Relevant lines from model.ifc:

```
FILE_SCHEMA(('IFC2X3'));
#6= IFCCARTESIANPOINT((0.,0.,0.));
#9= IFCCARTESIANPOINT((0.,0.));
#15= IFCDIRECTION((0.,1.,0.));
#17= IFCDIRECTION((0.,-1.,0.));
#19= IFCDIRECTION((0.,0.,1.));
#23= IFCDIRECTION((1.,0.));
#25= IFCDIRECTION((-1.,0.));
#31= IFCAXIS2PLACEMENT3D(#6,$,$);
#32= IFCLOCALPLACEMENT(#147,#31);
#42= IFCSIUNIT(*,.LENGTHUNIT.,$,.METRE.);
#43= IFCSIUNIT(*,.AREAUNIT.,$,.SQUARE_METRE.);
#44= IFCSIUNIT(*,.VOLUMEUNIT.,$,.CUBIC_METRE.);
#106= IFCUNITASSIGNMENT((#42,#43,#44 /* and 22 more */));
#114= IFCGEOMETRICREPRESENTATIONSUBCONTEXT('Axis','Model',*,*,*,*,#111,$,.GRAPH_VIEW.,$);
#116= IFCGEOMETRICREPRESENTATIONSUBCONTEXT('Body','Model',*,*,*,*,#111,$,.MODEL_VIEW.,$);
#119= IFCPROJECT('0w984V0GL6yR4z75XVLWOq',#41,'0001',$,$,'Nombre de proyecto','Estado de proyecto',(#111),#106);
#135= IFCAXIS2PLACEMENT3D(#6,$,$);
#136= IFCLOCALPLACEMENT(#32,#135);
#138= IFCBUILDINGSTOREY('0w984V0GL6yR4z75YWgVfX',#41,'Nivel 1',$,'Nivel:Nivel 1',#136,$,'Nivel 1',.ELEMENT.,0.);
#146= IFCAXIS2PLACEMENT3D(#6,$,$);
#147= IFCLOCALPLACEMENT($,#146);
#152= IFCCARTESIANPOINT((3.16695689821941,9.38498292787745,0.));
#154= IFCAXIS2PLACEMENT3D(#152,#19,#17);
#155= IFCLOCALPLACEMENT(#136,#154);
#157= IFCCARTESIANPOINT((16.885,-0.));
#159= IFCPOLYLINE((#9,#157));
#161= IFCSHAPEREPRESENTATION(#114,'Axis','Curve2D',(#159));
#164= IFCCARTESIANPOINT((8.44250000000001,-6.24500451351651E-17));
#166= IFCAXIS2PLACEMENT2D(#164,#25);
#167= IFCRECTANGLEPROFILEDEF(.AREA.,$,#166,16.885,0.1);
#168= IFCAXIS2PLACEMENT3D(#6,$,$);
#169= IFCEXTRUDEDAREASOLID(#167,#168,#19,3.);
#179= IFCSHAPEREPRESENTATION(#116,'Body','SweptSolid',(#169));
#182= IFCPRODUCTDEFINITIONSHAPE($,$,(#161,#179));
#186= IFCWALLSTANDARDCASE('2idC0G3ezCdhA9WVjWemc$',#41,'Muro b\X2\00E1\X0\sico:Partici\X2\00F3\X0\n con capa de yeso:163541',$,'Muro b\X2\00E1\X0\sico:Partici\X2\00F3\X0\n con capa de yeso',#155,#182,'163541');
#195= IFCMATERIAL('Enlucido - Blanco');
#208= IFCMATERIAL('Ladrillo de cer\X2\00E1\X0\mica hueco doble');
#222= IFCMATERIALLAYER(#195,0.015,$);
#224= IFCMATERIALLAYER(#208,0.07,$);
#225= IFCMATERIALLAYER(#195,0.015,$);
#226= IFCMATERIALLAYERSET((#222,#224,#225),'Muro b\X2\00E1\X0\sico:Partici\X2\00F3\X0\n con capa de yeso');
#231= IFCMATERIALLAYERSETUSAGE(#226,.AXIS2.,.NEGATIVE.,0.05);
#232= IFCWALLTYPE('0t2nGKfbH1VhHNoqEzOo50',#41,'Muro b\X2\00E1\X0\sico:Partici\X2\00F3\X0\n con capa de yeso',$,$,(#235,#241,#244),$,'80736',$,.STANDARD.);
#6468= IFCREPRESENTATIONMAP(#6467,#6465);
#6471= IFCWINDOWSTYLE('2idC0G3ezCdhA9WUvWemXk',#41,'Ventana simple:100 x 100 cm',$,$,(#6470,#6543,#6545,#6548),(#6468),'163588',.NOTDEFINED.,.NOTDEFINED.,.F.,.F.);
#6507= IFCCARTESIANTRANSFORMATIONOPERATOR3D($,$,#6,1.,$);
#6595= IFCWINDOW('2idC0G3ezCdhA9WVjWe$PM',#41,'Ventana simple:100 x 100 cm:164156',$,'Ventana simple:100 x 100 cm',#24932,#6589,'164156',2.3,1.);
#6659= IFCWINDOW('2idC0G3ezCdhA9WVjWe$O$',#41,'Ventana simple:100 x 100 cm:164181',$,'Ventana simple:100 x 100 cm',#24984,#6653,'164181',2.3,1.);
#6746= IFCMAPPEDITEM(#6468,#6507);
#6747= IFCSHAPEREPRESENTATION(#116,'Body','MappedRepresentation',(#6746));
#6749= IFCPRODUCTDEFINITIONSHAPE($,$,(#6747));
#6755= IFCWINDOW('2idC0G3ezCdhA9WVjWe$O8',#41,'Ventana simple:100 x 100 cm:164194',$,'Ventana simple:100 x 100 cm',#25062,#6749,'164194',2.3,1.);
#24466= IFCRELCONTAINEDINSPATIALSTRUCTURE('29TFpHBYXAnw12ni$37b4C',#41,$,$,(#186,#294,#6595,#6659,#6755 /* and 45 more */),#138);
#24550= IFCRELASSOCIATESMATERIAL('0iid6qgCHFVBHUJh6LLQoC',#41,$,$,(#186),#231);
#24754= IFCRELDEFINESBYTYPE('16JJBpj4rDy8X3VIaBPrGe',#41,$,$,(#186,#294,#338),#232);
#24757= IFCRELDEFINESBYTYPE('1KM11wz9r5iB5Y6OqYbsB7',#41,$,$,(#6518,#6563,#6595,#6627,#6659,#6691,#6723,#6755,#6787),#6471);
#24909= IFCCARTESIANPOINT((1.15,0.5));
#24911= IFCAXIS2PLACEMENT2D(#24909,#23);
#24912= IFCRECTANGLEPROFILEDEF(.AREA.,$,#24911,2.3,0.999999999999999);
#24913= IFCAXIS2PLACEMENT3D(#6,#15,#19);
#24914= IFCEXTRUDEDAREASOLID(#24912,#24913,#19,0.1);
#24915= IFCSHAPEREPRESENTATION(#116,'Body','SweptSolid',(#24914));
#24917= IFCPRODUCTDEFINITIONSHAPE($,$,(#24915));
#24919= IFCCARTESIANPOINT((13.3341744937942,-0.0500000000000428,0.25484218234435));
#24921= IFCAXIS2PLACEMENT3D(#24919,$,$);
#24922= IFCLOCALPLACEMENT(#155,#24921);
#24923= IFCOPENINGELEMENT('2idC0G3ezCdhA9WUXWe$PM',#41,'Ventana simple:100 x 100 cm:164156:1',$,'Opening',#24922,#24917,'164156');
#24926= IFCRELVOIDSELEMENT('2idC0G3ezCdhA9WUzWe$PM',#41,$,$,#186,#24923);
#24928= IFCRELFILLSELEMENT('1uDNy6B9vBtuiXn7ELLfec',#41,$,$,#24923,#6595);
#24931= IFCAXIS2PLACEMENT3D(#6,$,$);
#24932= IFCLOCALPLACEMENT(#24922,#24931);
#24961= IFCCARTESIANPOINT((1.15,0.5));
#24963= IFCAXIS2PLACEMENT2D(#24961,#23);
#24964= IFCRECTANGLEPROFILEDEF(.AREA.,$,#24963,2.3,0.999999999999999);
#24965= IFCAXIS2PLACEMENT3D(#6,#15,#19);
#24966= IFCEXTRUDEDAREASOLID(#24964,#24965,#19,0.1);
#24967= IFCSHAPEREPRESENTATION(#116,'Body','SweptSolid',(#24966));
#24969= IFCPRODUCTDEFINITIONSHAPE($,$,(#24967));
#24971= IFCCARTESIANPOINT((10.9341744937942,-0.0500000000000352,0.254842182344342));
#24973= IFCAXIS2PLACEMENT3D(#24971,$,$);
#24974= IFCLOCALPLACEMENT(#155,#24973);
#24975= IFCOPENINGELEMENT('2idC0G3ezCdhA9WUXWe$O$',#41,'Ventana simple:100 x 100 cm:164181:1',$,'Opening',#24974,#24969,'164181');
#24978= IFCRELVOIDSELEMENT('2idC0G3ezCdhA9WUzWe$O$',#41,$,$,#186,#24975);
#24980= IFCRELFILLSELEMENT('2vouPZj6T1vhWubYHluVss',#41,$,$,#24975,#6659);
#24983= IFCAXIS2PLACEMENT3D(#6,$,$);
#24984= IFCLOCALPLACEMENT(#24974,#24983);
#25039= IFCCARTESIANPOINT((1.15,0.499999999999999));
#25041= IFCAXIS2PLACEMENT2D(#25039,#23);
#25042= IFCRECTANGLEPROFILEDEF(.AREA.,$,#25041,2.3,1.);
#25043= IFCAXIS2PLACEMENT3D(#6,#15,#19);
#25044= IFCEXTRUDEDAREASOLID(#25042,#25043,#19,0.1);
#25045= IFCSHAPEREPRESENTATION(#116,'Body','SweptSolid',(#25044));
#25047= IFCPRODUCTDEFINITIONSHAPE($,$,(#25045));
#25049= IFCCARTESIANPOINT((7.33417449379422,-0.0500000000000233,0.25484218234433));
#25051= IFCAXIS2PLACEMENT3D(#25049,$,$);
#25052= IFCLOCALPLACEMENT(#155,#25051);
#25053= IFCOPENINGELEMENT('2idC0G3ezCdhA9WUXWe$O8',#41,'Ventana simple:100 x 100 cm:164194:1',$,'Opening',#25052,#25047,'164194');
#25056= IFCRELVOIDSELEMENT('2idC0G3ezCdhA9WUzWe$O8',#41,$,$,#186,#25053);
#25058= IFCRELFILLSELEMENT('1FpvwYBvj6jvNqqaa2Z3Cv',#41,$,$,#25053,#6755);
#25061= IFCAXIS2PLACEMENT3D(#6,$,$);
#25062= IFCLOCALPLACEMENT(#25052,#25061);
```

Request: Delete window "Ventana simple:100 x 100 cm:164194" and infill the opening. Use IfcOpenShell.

```python
import ifcopenshell
import ifcopenshell.api.feature
import ifcopenshell.api.root
import ifcopenshell.geom
import ifcopenshell.util.shape

model = ifcopenshell.open("model.ifc")
settings = ifcopenshell.geom.settings()


def volume(element):
    """Net volume in cubic metres, openings subtracted."""
    shape = ifcopenshell.geom.create_shape(settings, element)
    return ifcopenshell.util.shape.get_volume(shape.geometry)


window = model.by_guid("2idC0G3ezCdhA9WVjWe$O8")
opening = window.FillsVoids[0].RelatingOpeningElement
wall = opening.VoidsElements[0].RelatingBuildingElement
before = volume(wall)

ifcopenshell.api.root.remove_product(model, product=window)
ifcopenshell.api.feature.remove_feature(model, feature=opening)

after = volume(wall)

print(f"wall volume {before:.3f} -> {after:.3f} m3")

model.write("model_rev.ifc")
```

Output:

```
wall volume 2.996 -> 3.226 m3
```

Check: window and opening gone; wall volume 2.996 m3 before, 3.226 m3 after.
